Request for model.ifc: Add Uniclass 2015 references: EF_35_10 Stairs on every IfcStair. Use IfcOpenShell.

First a look at what the model holds.

```python
import ifcopenshell

model = ifcopenshell.open("model.ifc")
print(model.schema)
print("classifications:", [c.Name for c in model.by_type("IfcClassification")])
for ifc_class in ("IfcDoor", "IfcRoof", "IfcStair", "IfcWall", "IfcWindow"):
    print(ifc_class, len(model.by_type(ifc_class)))
```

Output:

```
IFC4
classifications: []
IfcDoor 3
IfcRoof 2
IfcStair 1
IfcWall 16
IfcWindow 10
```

```python
import ifcopenshell
import ifcopenshell.api.classification

model = ifcopenshell.open("model.ifc")

system = ifcopenshell.api.classification.add_classification(model, classification="Uniclass 2015")

codes = {
    "IfcStair": ("EF_35_10", "Stairs"),
}
for ifc_class, (code, name) in codes.items():
    products = model.by_type(ifc_class)
    ifcopenshell.api.classification.add_reference(
        model, products=products, classification=system, identification=code, name=name
    )
    print(code, len(products))

model.write("model-out.ifc")
```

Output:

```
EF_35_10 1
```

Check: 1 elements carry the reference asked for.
